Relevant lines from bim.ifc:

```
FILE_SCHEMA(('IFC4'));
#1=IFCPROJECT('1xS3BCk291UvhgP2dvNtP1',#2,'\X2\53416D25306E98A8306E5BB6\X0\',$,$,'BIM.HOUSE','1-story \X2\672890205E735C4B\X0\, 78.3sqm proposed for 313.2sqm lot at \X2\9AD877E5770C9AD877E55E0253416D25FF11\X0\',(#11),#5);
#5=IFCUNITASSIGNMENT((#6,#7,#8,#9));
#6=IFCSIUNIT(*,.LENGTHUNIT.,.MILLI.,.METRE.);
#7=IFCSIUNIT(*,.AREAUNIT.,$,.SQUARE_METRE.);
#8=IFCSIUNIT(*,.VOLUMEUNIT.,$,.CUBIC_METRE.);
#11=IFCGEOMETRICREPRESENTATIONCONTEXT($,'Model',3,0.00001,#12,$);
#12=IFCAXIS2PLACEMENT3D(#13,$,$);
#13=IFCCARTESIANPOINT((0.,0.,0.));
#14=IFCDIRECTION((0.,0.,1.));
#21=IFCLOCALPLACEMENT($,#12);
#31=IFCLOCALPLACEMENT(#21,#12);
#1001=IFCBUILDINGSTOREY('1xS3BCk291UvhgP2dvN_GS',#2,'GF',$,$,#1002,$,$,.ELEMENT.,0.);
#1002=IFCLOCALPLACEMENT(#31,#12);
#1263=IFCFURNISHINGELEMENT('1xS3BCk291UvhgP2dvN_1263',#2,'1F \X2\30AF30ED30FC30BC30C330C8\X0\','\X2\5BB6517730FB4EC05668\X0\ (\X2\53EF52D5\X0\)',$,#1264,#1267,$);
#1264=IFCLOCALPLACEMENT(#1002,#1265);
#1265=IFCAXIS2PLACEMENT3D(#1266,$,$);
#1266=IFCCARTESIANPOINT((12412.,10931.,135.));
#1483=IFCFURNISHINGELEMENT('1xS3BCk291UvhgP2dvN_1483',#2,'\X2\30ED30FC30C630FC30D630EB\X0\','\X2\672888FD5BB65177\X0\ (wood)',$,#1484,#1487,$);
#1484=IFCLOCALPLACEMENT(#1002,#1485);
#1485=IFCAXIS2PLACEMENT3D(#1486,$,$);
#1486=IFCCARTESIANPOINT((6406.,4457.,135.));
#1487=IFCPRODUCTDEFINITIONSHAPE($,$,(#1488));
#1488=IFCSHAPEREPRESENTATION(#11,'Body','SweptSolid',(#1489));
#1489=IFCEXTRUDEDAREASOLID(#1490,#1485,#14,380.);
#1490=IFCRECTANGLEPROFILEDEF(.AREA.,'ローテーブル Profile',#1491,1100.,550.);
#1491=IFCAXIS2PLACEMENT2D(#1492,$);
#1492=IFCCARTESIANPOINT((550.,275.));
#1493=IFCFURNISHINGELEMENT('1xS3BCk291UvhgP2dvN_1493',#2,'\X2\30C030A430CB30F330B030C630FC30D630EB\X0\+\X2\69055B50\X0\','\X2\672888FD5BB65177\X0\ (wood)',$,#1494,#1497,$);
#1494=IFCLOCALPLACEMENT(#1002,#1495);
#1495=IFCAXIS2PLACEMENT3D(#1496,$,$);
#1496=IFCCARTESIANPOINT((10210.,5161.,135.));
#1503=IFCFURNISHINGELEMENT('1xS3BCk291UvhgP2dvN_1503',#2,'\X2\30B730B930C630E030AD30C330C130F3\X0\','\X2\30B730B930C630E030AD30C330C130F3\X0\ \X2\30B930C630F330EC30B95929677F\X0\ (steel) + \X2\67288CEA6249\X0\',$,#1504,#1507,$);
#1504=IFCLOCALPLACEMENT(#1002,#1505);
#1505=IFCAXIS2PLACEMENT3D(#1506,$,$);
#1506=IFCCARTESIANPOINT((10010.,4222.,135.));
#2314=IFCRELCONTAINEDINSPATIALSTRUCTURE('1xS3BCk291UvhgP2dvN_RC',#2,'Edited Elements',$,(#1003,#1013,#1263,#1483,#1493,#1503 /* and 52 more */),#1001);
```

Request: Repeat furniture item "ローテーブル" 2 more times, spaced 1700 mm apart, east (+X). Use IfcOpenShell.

```python
import numpy as np
import ifcopenshell
import ifcopenshell.api.geometry
import ifcopenshell.api.root
import ifcopenshell.util.element
import ifcopenshell.util.placement
import ifcopenshell.util.unit

model = ifcopenshell.open("bim.ifc")
unit_scale = ifcopenshell.util.unit.calculate_unit_scale(model)


def reuse_history(source, copy):
    """copy_class also copies each property set's owner history, people and application; keep the originals."""
    for rel in copy.IsDefinedBy:
        if rel.is_a("IfcRelDefinesByProperties") and (history := rel.RelatingPropertyDefinition.OwnerHistory):
            rel.RelatingPropertyDefinition.OwnerHistory = source.OwnerHistory
            ifcopenshell.util.element.remove_deep2(model, history)


source = model.by_guid("1xS3BCk291UvhgP2dvN_1483")
base = ifcopenshell.util.placement.get_local_placement(source.ObjectPlacement)
step = np.array([1.0, 0.0, 0.0]) * 1.7 / unit_scale

for i in range(1, 3):
    copy = ifcopenshell.api.root.copy_class(model, product=source)
    copy.Representation = ifcopenshell.util.element.copy_deep(
        model, source.Representation, exclude=["IfcGeometricRepresentationContext", "IfcRepresentationMap"]
    )
    reuse_history(source, copy)
    matrix = base.copy()
    matrix[:3, 3] += i * step
    print("added at", matrix[:3, 3].round(3) + 0.0)
    ifcopenshell.api.geometry.edit_object_placement(model, product=copy, matrix=matrix, is_si=False)

model.write("bim_rev.ifc")
```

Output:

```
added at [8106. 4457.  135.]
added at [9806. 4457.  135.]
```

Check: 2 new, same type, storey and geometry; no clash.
